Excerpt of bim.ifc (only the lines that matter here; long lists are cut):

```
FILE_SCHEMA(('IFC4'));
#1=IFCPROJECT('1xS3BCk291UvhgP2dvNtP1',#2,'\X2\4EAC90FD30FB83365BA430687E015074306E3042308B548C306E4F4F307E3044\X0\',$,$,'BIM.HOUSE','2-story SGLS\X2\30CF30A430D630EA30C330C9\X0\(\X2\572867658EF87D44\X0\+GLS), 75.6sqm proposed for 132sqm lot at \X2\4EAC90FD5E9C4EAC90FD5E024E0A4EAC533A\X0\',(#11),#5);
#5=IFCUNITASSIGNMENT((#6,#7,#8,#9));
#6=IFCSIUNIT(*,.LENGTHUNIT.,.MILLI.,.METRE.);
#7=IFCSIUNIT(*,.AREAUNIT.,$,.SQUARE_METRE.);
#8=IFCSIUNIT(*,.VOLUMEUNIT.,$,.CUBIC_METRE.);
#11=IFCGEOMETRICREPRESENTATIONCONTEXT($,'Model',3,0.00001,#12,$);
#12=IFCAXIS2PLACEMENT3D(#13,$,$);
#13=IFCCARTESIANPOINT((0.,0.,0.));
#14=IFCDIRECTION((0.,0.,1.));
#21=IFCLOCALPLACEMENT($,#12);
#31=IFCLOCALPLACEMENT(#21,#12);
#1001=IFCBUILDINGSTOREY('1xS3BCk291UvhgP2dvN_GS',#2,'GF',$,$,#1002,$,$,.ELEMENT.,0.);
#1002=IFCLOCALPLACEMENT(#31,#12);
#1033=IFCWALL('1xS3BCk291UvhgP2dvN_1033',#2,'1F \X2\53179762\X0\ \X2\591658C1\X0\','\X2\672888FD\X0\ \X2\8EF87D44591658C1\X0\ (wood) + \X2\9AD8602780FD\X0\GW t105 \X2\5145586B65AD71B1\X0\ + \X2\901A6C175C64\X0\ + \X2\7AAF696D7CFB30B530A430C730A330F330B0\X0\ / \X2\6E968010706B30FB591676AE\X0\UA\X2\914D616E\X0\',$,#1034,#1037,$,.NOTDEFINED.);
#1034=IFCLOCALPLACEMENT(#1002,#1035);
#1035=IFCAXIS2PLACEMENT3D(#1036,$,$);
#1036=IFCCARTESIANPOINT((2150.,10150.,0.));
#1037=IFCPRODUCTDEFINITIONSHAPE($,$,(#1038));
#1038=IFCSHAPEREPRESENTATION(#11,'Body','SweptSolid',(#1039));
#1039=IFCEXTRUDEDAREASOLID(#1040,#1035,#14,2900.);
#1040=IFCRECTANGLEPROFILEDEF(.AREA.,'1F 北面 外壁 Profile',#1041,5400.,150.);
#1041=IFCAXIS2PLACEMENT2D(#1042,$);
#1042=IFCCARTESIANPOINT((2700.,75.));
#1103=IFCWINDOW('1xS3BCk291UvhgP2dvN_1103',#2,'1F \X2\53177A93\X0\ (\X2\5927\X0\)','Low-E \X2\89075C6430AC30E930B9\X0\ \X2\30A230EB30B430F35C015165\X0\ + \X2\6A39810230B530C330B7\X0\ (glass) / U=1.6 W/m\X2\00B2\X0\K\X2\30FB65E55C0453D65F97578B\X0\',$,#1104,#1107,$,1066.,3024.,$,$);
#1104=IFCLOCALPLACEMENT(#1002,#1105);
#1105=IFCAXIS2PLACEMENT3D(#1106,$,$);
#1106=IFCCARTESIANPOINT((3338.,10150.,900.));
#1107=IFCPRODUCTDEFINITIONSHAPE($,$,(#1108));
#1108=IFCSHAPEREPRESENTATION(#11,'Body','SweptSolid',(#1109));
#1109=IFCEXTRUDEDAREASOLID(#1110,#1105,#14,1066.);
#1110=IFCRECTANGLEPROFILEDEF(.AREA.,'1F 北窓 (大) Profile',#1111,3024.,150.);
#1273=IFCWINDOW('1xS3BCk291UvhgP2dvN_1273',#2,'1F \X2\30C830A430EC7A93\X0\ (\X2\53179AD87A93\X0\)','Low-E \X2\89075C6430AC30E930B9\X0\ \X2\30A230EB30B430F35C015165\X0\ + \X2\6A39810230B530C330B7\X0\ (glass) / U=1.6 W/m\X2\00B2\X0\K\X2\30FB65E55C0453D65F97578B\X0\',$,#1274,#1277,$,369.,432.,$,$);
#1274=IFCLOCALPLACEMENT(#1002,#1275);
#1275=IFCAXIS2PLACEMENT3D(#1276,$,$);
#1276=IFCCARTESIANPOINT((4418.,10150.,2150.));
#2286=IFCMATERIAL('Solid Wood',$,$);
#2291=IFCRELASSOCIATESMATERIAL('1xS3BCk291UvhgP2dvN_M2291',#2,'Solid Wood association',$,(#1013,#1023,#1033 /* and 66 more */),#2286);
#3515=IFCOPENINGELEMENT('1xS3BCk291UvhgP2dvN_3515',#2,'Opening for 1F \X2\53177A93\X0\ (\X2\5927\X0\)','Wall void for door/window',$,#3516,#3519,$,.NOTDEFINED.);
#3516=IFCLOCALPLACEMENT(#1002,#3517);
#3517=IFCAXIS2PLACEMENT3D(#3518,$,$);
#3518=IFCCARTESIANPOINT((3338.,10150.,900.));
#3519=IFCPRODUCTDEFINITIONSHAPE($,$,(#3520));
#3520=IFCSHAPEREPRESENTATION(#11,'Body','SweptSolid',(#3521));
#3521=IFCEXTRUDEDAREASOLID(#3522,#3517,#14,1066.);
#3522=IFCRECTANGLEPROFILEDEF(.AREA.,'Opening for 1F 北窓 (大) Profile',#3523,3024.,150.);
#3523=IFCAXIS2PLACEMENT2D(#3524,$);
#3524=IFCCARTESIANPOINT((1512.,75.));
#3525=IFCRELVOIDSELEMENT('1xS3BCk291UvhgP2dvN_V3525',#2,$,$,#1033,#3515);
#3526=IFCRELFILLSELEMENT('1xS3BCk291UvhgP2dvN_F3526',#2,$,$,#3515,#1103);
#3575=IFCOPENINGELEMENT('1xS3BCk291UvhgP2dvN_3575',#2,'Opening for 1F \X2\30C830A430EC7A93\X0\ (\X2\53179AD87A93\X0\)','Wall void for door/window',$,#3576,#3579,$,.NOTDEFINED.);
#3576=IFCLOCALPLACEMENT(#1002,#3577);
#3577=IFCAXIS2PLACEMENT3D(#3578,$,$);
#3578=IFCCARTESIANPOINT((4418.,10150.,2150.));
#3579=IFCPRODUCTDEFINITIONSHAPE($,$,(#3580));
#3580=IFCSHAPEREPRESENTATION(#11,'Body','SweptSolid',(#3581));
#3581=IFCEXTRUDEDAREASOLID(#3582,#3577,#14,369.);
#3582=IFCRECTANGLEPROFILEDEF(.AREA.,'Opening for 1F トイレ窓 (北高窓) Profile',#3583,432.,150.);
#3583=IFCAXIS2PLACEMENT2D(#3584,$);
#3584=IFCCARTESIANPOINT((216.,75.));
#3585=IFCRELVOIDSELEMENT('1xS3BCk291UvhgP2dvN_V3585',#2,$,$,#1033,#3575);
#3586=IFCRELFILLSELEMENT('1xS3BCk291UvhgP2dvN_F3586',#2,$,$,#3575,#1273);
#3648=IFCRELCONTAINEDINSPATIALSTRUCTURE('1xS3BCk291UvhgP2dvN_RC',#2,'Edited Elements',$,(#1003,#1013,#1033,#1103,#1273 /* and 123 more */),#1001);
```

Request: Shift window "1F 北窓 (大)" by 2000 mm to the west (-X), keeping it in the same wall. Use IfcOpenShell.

```python
import ifcopenshell
import ifcopenshell.api.geometry
import ifcopenshell.util.placement
import ifcopenshell.util.unit

model = ifcopenshell.open("bim.ifc")
unit_scale = ifcopenshell.util.unit.calculate_unit_scale(model)

window = model.by_guid("1xS3BCk291UvhgP2dvN_1103")
opening = window.FillsVoids[0].RelatingOpeningElement
wall = opening.VoidsElements[0].RelatingBuildingElement

wall_matrix = ifcopenshell.util.placement.get_local_placement(wall.ObjectPlacement)
shift = wall_matrix[:3, 0] * -2 / unit_scale
before = ifcopenshell.util.placement.get_local_placement(window.ObjectPlacement)[:3, 3].copy()

# The window is not placed relative to its opening, so move both.
for product in (opening, window):
    matrix = ifcopenshell.util.placement.get_local_placement(product.ObjectPlacement)
    matrix[:3, 3] += shift
    ifcopenshell.api.geometry.edit_object_placement(model, product=product, matrix=matrix, is_si=False)

after = ifcopenshell.util.placement.get_local_placement(window.ObjectPlacement)[:3, 3]
print("window moved by", (after - before).round(3) + 0.0)

model.write("bim_v2.ifc")
```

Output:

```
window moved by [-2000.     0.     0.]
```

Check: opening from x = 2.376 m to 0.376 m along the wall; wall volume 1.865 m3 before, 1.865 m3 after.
